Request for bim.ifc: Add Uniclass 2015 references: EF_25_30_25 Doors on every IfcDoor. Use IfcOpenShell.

First a look at what the model holds.

```python
import ifcopenshell

model = ifcopenshell.open("bim.ifc")
print(model.schema)
print("classifications:", [c.Name for c in model.by_type("IfcClassification")])
for ifc_class in ("IfcDoor", "IfcRoof", "IfcStair", "IfcWall", "IfcWindow"):
    print(ifc_class, len(model.by_type(ifc_class)))
```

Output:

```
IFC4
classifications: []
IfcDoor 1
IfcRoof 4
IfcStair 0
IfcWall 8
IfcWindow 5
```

```python
import ifcopenshell
import ifcopenshell.api.classification

model = ifcopenshell.open("bim.ifc")

system = ifcopenshell.api.classification.add_classification(model, classification="Uniclass 2015")

codes = {
    "IfcDoor": ("EF_25_30_25", "Doors"),
}
for ifc_class, (code, name) in codes.items():
    products = model.by_type(ifc_class)
    ifcopenshell.api.classification.add_reference(
        model, products=products, classification=system, identification=code, name=name
    )
    print(code, len(products))

model.write("bim-out.ifc")
```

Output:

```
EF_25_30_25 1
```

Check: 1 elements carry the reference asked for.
